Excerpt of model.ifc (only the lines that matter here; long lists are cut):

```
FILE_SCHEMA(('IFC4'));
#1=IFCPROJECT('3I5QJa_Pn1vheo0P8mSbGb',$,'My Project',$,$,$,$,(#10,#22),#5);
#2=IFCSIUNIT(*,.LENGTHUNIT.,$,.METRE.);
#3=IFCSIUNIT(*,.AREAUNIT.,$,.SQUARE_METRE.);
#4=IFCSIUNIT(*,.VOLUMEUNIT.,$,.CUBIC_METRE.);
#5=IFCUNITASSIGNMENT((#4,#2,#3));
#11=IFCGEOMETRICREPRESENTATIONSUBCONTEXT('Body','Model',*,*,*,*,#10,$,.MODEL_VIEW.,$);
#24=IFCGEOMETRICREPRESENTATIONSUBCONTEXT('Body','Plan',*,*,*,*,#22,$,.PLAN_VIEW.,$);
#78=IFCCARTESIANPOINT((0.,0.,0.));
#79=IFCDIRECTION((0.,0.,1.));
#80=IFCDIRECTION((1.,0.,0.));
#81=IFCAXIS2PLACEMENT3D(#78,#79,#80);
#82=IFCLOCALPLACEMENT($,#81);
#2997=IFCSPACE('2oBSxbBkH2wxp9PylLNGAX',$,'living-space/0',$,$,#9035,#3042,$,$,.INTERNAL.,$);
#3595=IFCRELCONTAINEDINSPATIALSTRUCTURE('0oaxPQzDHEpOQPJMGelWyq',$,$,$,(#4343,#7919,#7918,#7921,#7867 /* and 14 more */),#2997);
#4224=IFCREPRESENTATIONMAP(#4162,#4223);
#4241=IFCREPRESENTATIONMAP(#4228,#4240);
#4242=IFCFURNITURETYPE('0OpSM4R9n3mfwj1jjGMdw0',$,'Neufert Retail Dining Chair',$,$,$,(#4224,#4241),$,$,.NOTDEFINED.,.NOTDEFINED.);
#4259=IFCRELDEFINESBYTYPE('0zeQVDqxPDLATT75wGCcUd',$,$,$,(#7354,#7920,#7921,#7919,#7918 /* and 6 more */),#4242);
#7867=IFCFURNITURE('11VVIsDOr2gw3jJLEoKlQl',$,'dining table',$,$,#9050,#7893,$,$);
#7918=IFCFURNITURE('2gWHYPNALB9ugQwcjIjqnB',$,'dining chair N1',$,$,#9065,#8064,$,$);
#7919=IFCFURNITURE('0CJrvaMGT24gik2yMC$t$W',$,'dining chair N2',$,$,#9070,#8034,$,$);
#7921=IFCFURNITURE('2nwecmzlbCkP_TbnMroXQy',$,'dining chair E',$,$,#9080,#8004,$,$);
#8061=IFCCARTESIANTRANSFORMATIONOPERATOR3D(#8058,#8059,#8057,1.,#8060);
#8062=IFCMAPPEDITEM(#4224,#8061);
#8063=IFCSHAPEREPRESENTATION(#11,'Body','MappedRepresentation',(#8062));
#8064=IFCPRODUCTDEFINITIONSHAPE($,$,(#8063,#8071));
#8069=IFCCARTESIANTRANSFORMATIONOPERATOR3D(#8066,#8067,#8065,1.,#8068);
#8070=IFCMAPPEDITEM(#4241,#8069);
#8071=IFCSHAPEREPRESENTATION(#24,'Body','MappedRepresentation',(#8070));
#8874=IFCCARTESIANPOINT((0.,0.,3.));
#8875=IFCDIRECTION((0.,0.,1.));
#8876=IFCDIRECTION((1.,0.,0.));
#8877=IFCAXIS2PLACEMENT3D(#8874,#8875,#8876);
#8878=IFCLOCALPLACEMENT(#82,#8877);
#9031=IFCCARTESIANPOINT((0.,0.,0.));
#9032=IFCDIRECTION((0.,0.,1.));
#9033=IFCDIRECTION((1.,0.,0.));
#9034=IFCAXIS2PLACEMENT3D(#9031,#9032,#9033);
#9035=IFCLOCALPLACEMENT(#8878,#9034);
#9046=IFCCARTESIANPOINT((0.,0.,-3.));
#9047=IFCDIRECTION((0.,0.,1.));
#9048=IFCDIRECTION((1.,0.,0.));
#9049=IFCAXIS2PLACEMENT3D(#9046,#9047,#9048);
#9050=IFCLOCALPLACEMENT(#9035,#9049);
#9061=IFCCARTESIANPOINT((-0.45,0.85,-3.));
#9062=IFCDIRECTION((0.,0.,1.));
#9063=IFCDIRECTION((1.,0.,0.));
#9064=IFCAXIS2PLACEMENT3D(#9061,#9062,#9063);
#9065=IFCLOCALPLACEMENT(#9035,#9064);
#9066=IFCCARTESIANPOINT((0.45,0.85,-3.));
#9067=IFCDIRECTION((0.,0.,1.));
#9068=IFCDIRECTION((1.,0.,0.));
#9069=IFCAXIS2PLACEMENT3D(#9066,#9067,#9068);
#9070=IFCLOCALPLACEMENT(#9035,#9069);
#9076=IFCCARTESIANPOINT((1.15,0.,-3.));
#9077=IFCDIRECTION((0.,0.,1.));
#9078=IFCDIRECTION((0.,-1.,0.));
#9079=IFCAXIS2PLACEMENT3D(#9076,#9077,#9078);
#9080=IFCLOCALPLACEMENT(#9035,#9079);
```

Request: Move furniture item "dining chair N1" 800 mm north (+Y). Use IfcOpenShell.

```python
import ifcopenshell
import ifcopenshell.api.geometry
import ifcopenshell.util.placement
import ifcopenshell.util.unit

model = ifcopenshell.open("model.ifc")
unit_scale = ifcopenshell.util.unit.calculate_unit_scale(model)

item = model.by_guid("2gWHYPNALB9ugQwcjIjqnB")
matrix = ifcopenshell.util.placement.get_local_placement(item.ObjectPlacement)
matrix[1, 3] += 0.8 / unit_scale
ifcopenshell.api.geometry.edit_object_placement(model, product=item, matrix=matrix, is_si=False)

print(ifcopenshell.util.placement.get_local_placement(item.ObjectPlacement).round(3) + 0.0)

model.write("model_rev.ifc")
```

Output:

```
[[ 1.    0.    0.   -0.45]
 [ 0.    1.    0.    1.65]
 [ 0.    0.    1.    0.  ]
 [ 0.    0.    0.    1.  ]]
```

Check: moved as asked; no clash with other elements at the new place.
